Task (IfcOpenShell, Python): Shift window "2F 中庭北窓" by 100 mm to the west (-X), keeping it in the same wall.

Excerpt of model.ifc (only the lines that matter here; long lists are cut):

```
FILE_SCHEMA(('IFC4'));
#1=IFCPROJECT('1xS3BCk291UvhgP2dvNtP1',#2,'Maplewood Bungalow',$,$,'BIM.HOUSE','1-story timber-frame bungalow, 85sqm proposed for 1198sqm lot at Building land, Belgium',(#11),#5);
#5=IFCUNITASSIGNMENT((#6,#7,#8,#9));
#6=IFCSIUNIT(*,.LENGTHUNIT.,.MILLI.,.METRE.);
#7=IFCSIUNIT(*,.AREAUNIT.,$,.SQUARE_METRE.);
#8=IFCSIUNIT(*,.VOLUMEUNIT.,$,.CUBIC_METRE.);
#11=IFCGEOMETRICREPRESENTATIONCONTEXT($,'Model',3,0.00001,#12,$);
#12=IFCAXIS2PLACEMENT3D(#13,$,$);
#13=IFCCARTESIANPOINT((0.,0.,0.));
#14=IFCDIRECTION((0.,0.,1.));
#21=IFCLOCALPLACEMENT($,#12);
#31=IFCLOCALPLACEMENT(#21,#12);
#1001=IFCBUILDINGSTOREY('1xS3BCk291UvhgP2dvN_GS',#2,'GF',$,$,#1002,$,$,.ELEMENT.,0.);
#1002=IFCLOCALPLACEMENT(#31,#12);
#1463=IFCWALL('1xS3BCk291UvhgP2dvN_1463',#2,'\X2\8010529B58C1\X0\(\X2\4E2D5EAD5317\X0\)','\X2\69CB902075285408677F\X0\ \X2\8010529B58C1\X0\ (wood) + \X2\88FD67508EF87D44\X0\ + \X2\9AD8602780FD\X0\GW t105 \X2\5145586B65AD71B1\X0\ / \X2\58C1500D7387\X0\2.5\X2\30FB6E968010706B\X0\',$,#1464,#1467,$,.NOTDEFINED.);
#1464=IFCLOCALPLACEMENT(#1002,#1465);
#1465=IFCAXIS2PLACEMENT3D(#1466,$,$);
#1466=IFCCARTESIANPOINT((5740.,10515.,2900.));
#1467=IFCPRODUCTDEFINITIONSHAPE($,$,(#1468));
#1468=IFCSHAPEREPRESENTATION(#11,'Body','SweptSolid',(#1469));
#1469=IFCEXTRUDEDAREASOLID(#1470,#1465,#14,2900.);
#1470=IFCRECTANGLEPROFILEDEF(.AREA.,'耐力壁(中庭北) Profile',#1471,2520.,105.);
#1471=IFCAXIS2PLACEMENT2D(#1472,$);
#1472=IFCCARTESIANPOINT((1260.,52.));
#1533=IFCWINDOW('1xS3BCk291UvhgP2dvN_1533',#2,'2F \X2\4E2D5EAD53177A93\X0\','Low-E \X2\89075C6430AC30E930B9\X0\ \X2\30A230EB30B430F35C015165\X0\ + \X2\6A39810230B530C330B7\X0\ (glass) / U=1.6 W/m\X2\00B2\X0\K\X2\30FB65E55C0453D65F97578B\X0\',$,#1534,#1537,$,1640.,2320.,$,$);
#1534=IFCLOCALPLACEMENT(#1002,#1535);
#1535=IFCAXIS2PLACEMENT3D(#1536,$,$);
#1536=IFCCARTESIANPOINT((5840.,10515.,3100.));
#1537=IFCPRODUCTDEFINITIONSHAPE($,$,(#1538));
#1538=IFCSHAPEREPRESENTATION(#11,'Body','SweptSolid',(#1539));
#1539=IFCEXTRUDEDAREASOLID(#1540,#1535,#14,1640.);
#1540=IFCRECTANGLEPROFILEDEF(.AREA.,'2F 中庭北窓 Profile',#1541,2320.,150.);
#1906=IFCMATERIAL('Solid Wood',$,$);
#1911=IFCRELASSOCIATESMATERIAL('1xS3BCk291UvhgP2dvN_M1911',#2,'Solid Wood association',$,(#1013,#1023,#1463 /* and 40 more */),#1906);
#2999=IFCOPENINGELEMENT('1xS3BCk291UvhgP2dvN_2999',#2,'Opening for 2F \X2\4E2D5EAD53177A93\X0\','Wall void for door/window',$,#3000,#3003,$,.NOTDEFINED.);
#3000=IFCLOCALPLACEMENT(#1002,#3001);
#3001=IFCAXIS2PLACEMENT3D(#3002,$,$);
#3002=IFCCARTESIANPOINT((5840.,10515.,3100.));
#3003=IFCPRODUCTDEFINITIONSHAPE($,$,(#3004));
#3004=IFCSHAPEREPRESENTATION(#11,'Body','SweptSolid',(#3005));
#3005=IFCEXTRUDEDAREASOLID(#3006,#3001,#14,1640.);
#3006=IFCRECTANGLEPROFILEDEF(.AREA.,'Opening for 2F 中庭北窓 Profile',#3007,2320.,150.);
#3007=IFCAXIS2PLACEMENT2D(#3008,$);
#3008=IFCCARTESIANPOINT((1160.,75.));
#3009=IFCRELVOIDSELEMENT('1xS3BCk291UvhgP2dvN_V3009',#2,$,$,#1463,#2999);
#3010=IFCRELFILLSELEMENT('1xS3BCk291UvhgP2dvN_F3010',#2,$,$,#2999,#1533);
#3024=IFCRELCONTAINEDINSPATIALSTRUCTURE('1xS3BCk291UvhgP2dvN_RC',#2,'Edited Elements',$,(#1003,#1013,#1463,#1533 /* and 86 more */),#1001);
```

```python
import ifcopenshell
import ifcopenshell.api.geometry
import ifcopenshell.util.placement
import ifcopenshell.util.unit

model = ifcopenshell.open("model.ifc")
unit_scale = ifcopenshell.util.unit.calculate_unit_scale(model)

window = model.by_id(1533)
opening = window.FillsVoids[0].RelatingOpeningElement
wall = opening.VoidsElements[0].RelatingBuildingElement

wall_matrix = ifcopenshell.util.placement.get_local_placement(wall.ObjectPlacement)
shift = wall_matrix[:3, 0] * -0.1 / unit_scale
before = ifcopenshell.util.placement.get_local_placement(window.ObjectPlacement)[:3, 3].copy()

# The window is not placed relative to its opening, so move both.
for product in (opening, window):
    matrix = ifcopenshell.util.placement.get_local_placement(product.ObjectPlacement)
    matrix[:3, 3] += shift
    ifcopenshell.api.geometry.edit_object_placement(model, product=product, matrix=matrix, is_si=False)

after = ifcopenshell.util.placement.get_local_placement(window.ObjectPlacement)[:3, 3]
print("window moved by", (after - before).round(3) + 0.0)

model.write("model_updated.ifc")
```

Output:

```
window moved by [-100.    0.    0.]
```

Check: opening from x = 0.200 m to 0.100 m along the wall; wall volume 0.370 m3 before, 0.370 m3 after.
